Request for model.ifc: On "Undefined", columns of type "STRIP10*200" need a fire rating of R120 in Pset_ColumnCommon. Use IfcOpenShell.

First a look at what the model holds.

```python
import ifcopenshell
import ifcopenshell.util.element

model = ifcopenshell.open("model.ifc")
print(model.schema)
storey = next(s for s in model.by_type("IfcBuildingStorey") if s.Name == "Undefined")
columns = [e for e in ifcopenshell.util.element.get_decomposition(storey) if e.is_a("IfcColumn")]
seen = {}
for e in columns:
    element_type = ifcopenshell.util.element.get_type(e)
    key = (element_type.Name if element_type != e and element_type else None, ifcopenshell.util.element.get_pset(e, "Pset_ColumnCommon", "FireRating"))
    seen[key] = seen.get(key, 0) + 1
for (name, value), count in sorted(seen.items(), key=str):
    print(count, "x", name, "|", value)
```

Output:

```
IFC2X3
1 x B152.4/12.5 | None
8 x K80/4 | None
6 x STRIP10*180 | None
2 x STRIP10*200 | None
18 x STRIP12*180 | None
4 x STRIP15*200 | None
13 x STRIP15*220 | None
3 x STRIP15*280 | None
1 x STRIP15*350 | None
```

```python
import ifcopenshell
import ifcopenshell.api.pset
import ifcopenshell.util.element

model = ifcopenshell.open("model.ifc")

storey = next(s for s in model.by_type("IfcBuildingStorey") if s.Name == "Undefined")
columns = [e for e in ifcopenshell.util.element.get_decomposition(storey) if e.is_a("IfcColumn")]

count = 0
for e in columns:
    element_type = ifcopenshell.util.element.get_type(e)
    if element_type in (None, e) or element_type.Name != "STRIP10*200":
        continue
    # add_pset returns the element's existing set when there is one.
    pset = ifcopenshell.api.pset.add_pset(model, product=e, name="Pset_ColumnCommon")
    ifcopenshell.api.pset.edit_pset(model, pset=pset, properties={"FireRating": "R120"})
    count += 1

print(count, "columns updated")

model.write("model-out.ifc")
```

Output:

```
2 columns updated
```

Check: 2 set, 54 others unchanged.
